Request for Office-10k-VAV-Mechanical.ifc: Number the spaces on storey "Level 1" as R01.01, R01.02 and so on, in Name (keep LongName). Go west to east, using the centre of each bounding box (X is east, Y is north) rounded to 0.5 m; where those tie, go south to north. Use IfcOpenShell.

First a look at what the model holds.

```python
import ifcopenshell
import ifcopenshell.util.element
import ifcopenshell.util.placement

model = ifcopenshell.open("Office-10k-VAV-Mechanical.ifc")
print(model.schema)
storey = next(s for s in model.by_type("IfcBuildingStorey") if s.Name == "Level 1")
spaces = [e for e in ifcopenshell.util.element.get_decomposition(storey) if e.is_a("IfcSpace")]
for e in sorted(spaces, key=lambda e: e.id()):
    origin = ifcopenshell.util.placement.get_local_placement(e.ObjectPlacement)[:3, 3]
    print(e.id(), e.Name, e.LongName, origin.round(2) + 0.0, sep=" | ")
```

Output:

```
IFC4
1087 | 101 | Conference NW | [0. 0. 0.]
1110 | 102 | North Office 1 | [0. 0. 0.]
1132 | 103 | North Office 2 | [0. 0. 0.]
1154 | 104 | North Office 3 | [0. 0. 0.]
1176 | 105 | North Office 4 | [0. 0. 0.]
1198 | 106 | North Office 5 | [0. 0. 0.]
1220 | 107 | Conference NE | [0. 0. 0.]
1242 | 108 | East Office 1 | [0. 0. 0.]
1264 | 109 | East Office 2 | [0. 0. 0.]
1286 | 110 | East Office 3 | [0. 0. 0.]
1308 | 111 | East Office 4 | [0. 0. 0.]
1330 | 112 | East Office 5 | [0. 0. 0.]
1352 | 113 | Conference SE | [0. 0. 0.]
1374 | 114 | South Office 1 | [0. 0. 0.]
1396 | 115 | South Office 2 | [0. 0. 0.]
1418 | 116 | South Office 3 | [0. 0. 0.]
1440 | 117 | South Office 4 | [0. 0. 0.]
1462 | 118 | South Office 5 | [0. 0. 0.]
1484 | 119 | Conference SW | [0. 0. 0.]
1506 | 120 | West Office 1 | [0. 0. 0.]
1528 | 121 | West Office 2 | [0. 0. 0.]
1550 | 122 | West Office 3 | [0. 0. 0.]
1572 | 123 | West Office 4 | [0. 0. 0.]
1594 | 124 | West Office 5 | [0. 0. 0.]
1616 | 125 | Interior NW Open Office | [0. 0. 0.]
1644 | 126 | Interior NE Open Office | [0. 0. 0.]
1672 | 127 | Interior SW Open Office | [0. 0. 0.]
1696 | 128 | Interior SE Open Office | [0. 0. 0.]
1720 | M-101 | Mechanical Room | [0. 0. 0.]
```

```python
import ifcopenshell
import ifcopenshell.geom
import ifcopenshell.util.element
import ifcopenshell.util.shape

model = ifcopenshell.open("Office-10k-VAV-Mechanical.ifc")
settings = ifcopenshell.geom.settings()
settings.set("use-world-coords", True)


def centre(element):
    shape = ifcopenshell.geom.create_shape(settings, element)
    return ifcopenshell.util.shape.get_bbox_centroid(shape.geometry)


storey = next(s for s in model.by_type("IfcBuildingStorey") if s.Name == "Level 1")
spaces = [e for e in ifcopenshell.util.element.get_decomposition(storey) if e.is_a("IfcSpace")]

# Insertion points can sit at a corner or the storey origin, so sort by the geometry (in metres).
centres = {e: centre(e) for e in spaces}
spaces.sort(key=lambda e: (round(centres[e][0] / 0.5), centres[e][1]))

for i, e in enumerate(spaces, start=1):
    number = f"R01.{i:02d}"
    e.Name = number
    print(e.id(), number)

model.write("Office-10k-VAV-Mechanical_rev.ifc")
```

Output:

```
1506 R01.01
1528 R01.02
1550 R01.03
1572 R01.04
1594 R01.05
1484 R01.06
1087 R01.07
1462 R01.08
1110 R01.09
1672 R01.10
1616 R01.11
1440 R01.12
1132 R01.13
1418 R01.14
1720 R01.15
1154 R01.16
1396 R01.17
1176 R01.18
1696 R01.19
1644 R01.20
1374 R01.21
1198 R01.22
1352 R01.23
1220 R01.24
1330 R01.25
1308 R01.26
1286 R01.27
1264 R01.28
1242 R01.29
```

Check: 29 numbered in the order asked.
